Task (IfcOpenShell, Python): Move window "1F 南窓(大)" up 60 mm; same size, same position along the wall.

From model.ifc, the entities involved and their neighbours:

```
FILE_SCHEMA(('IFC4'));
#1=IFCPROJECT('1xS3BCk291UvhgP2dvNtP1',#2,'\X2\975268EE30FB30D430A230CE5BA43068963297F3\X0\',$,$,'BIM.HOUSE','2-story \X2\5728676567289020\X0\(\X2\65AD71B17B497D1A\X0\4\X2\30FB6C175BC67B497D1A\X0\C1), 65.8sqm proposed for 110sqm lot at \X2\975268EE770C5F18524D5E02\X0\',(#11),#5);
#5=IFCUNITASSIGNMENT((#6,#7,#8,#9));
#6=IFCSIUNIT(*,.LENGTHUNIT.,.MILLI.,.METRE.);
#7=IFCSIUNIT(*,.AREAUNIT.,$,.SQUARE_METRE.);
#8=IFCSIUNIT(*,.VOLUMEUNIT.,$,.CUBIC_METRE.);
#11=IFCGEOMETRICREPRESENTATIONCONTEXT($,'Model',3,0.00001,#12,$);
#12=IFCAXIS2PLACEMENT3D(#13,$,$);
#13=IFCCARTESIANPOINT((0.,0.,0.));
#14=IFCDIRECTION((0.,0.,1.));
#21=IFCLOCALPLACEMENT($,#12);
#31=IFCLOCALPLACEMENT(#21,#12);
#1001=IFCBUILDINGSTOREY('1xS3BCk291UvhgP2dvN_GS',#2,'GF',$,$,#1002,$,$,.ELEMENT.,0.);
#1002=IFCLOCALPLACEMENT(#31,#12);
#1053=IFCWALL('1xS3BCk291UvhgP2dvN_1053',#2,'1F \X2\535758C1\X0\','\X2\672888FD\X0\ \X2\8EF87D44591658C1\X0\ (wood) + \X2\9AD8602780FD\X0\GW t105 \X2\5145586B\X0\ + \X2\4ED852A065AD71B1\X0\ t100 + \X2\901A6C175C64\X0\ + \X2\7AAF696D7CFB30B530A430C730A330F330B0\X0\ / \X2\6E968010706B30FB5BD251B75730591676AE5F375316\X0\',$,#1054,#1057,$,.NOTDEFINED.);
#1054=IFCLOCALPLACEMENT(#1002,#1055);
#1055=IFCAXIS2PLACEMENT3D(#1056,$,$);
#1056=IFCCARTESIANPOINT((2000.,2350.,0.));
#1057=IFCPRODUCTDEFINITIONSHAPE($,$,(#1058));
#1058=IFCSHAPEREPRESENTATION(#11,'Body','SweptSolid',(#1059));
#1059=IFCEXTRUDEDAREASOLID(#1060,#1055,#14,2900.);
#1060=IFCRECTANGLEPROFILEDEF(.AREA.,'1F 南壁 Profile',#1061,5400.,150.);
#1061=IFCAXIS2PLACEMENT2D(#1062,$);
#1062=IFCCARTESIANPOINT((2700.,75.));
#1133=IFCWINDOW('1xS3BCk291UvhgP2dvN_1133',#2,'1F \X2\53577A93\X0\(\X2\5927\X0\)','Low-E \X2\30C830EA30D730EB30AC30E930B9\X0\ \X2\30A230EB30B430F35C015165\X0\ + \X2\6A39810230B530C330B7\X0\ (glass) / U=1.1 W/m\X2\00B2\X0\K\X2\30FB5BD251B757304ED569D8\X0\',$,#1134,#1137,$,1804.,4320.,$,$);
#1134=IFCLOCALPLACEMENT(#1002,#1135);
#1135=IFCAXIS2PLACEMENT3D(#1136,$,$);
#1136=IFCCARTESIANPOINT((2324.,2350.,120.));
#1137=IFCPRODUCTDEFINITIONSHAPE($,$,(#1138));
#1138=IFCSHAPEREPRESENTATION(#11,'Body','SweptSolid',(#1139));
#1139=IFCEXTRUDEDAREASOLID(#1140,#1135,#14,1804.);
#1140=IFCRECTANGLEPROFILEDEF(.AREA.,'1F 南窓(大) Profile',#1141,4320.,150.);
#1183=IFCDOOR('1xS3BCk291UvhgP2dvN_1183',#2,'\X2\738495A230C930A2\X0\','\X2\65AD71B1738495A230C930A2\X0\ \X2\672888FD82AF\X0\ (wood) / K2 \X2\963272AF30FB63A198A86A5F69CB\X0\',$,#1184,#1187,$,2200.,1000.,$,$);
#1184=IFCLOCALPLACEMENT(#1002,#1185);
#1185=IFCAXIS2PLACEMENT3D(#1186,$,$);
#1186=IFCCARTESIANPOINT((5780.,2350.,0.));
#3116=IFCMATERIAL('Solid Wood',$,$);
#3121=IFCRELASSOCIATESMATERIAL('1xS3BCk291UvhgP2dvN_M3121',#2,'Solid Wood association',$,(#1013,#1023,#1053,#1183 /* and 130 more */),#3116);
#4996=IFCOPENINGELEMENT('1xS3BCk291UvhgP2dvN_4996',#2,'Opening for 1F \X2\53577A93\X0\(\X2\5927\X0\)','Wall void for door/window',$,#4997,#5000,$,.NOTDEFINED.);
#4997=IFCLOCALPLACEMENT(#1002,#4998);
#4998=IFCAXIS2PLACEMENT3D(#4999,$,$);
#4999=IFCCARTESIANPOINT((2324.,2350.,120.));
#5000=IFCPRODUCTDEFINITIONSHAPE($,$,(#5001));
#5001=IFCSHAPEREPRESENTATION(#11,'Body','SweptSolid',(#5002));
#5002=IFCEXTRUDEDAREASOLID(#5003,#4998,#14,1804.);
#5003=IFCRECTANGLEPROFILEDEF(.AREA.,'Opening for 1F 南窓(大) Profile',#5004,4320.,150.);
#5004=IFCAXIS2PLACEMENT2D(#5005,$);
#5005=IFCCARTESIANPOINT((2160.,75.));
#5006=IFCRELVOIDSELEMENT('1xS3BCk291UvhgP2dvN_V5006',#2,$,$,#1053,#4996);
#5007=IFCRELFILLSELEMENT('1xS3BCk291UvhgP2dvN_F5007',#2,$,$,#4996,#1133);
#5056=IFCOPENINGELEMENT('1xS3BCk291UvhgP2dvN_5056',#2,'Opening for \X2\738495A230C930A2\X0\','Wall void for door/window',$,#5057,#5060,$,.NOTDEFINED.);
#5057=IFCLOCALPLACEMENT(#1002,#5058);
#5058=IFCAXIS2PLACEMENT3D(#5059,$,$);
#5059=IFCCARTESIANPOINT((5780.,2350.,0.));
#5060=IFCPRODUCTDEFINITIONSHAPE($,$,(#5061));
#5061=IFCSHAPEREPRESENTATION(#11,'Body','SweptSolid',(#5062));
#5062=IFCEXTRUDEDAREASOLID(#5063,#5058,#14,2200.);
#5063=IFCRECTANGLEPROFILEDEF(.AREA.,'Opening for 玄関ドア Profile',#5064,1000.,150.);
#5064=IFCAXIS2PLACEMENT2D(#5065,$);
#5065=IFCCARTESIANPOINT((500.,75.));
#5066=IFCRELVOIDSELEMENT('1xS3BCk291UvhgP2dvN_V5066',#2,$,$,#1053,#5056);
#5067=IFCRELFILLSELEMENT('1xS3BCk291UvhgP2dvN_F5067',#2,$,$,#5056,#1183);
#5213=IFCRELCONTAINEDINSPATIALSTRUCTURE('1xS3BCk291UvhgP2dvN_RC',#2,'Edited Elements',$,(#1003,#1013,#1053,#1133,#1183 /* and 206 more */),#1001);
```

```python
import numpy as np
import ifcopenshell
import ifcopenshell.api.geometry
import ifcopenshell.util.placement
import ifcopenshell.util.unit

model = ifcopenshell.open("model.ifc")
unit_scale = ifcopenshell.util.unit.calculate_unit_scale(model)

window = model.by_id(1133)
opening = window.FillsVoids[0].RelatingOpeningElement
dz = 0.06 / unit_scale

shift = np.array([0.0, 0.0, dz])
# The window is not placed relative to its opening, so move both.
for product in (opening, window):
    matrix = ifcopenshell.util.placement.get_local_placement(product.ObjectPlacement)
    matrix[:3, 3] += shift
    ifcopenshell.api.geometry.edit_object_placement(model, product=product, matrix=matrix, is_si=False)

print(f"moved by {dz * unit_scale:+.3f} m")

model.write("model_edited.ifc")
```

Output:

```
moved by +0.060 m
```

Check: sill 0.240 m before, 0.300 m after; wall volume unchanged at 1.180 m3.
